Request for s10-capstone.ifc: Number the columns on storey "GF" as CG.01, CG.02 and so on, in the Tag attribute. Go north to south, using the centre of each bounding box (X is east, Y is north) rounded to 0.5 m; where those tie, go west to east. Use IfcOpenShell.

First a look at what the model holds.

```python
import ifcopenshell
import ifcopenshell.util.element
import ifcopenshell.util.placement

model = ifcopenshell.open("s10-capstone.ifc")
print(model.schema)
storey = next(s for s in model.by_type("IfcBuildingStorey") if s.Name == "GF")
columns = [e for e in ifcopenshell.util.element.get_decomposition(storey) if e.is_a("IfcColumn")]
for e in sorted(columns, key=lambda e: e.id()):
    origin = ifcopenshell.util.placement.get_local_placement(e.ObjectPlacement)[:3, 3]
    print(e.id(), e.Tag, e.Name, origin.round(2) + 0.0, sep=" | ")
```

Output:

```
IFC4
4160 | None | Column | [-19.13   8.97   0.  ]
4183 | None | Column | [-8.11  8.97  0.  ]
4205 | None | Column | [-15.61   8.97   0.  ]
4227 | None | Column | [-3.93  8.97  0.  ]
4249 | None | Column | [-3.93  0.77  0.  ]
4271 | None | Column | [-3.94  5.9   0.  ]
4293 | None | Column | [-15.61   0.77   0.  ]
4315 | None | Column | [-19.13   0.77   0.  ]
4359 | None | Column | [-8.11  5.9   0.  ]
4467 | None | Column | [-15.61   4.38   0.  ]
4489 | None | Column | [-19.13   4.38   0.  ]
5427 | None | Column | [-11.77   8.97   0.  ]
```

```python
import ifcopenshell
import ifcopenshell.geom
import ifcopenshell.util.element
import ifcopenshell.util.shape

model = ifcopenshell.open("s10-capstone.ifc")
settings = ifcopenshell.geom.settings()
settings.set("use-world-coords", True)


def centre(element):
    shape = ifcopenshell.geom.create_shape(settings, element)
    return ifcopenshell.util.shape.get_bbox_centroid(shape.geometry)


storey = next(s for s in model.by_type("IfcBuildingStorey") if s.Name == "GF")
columns = [e for e in ifcopenshell.util.element.get_decomposition(storey) if e.is_a("IfcColumn")]

# Insertion points can sit at a corner or the storey origin, so sort by the geometry (in metres).
centres = {e: centre(e) for e in columns}
columns.sort(key=lambda e: (-round(centres[e][1] / 0.5), centres[e][0]))

for i, e in enumerate(columns, start=1):
    number = f"CG.{i:02d}"
    e.Tag = number
    print(e.id(), number)

model.write("s10-capstone_updated.ifc")
```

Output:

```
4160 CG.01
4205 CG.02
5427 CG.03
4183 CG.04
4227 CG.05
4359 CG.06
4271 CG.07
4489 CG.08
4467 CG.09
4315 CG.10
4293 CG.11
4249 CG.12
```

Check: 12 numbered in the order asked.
